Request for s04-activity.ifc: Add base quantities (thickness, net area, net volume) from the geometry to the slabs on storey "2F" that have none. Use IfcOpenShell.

First a look at what the model holds.

```python
import ifcopenshell
import ifcopenshell.util.element
import ifcopenshell.util.unit

model = ifcopenshell.open("s04-activity.ifc")
print(model.schema)
for unit_type in ("LENGTHUNIT", "AREAUNIT", "VOLUMEUNIT"):
    print(unit_type, ifcopenshell.util.unit.calculate_unit_scale(model, unit_type))
storey = next(s for s in model.by_type("IfcBuildingStorey") if s.Name == "2F")
slabs = [e for e in ifcopenshell.util.element.get_decomposition(storey) if e.is_a("IfcSlab")]
for e in sorted(slabs, key=lambda e: e.id()):
    print(e.id(), e.is_a(), e.Name, list(ifcopenshell.util.element.get_psets(e, qtos_only=True)), sep=" | ")
```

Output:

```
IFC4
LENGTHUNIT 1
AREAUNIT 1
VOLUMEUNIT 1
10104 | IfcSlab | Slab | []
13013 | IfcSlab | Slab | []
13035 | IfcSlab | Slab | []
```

```python
import ifcopenshell
import ifcopenshell.api.pset
import ifcopenshell.geom
import ifcopenshell.util.element
import ifcopenshell.util.shape
import ifcopenshell.util.unit

model = ifcopenshell.open("s04-activity.ifc")
unit_scale = ifcopenshell.util.unit.calculate_unit_scale(model)
area_scale = ifcopenshell.util.unit.calculate_unit_scale(model, "AREAUNIT")
volume_scale = ifcopenshell.util.unit.calculate_unit_scale(model, "VOLUMEUNIT")
settings = ifcopenshell.geom.settings()

storey = next(s for s in model.by_type("IfcBuildingStorey") if s.Name == "2F")
slabs = [e for e in ifcopenshell.util.element.get_decomposition(storey) if e.is_a("IfcSlab")]

for e in sorted(slabs, key=lambda e: e.id()):
    if ifcopenshell.util.element.get_psets(e, qtos_only=True, should_inherit=False):
        continue
    # Geometry comes back in metres, in the element's own axes.
    shape = ifcopenshell.geom.create_shape(settings, e)
    values = {
        "Width": ifcopenshell.util.shape.get_z(shape.geometry) / unit_scale,
        "NetArea": ifcopenshell.util.shape.get_footprint_area(shape.geometry) / area_scale,
        "NetVolume": ifcopenshell.util.shape.get_volume(shape.geometry) / volume_scale,
    }
    qto = ifcopenshell.api.pset.add_qto(model, product=e, name="Qto_SlabBaseQuantities")
    ifcopenshell.api.pset.edit_qto(model, qto=qto, properties=values)
    print(e.id(), {k: round(v, 3) for k, v in values.items()})

model.write("s04-activity_edited.ifc")
```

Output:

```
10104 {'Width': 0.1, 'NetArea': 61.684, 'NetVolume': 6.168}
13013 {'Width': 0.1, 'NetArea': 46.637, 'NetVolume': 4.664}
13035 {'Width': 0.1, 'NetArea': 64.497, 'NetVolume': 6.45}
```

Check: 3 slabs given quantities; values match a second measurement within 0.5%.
